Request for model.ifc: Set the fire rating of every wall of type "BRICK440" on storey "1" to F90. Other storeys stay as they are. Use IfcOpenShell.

First a look at what the model holds.

```python
import ifcopenshell
import ifcopenshell.util.element

model = ifcopenshell.open("model.ifc")
print(model.schema)
storey = next(s for s in model.by_type("IfcBuildingStorey") if s.Name == "1")
walls = [e for e in ifcopenshell.util.element.get_decomposition(storey) if e.is_a("IfcWall")]
seen = {}
for e in walls:
    element_type = ifcopenshell.util.element.get_type(e)
    key = (element_type.Name if element_type != e and element_type else None, ifcopenshell.util.element.get_pset(e, "Pset_WallCommon", "FireRating"))
    seen[key] = seen.get(key, 0) + 1
for (name, value), count in sorted(seen.items(), key=str):
    print(count, "x", name, "|", value)
```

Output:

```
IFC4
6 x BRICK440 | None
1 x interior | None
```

```python
import ifcopenshell
import ifcopenshell.api.pset
import ifcopenshell.util.element

model = ifcopenshell.open("model.ifc")

storey = next(s for s in model.by_type("IfcBuildingStorey") if s.Name == "1")
walls = [e for e in ifcopenshell.util.element.get_decomposition(storey) if e.is_a("IfcWall")]

count = 0
for e in walls:
    element_type = ifcopenshell.util.element.get_type(e)
    if element_type in (None, e) or element_type.Name != "BRICK440":
        continue
    # add_pset returns the element's existing set when there is one.
    pset = ifcopenshell.api.pset.add_pset(model, product=e, name="Pset_WallCommon")
    ifcopenshell.api.pset.edit_pset(model, pset=pset, properties={"FireRating": "F90"})
    count += 1

print(count, "walls updated")

model.write("model_v2.ifc")
```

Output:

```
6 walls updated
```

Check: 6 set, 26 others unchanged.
